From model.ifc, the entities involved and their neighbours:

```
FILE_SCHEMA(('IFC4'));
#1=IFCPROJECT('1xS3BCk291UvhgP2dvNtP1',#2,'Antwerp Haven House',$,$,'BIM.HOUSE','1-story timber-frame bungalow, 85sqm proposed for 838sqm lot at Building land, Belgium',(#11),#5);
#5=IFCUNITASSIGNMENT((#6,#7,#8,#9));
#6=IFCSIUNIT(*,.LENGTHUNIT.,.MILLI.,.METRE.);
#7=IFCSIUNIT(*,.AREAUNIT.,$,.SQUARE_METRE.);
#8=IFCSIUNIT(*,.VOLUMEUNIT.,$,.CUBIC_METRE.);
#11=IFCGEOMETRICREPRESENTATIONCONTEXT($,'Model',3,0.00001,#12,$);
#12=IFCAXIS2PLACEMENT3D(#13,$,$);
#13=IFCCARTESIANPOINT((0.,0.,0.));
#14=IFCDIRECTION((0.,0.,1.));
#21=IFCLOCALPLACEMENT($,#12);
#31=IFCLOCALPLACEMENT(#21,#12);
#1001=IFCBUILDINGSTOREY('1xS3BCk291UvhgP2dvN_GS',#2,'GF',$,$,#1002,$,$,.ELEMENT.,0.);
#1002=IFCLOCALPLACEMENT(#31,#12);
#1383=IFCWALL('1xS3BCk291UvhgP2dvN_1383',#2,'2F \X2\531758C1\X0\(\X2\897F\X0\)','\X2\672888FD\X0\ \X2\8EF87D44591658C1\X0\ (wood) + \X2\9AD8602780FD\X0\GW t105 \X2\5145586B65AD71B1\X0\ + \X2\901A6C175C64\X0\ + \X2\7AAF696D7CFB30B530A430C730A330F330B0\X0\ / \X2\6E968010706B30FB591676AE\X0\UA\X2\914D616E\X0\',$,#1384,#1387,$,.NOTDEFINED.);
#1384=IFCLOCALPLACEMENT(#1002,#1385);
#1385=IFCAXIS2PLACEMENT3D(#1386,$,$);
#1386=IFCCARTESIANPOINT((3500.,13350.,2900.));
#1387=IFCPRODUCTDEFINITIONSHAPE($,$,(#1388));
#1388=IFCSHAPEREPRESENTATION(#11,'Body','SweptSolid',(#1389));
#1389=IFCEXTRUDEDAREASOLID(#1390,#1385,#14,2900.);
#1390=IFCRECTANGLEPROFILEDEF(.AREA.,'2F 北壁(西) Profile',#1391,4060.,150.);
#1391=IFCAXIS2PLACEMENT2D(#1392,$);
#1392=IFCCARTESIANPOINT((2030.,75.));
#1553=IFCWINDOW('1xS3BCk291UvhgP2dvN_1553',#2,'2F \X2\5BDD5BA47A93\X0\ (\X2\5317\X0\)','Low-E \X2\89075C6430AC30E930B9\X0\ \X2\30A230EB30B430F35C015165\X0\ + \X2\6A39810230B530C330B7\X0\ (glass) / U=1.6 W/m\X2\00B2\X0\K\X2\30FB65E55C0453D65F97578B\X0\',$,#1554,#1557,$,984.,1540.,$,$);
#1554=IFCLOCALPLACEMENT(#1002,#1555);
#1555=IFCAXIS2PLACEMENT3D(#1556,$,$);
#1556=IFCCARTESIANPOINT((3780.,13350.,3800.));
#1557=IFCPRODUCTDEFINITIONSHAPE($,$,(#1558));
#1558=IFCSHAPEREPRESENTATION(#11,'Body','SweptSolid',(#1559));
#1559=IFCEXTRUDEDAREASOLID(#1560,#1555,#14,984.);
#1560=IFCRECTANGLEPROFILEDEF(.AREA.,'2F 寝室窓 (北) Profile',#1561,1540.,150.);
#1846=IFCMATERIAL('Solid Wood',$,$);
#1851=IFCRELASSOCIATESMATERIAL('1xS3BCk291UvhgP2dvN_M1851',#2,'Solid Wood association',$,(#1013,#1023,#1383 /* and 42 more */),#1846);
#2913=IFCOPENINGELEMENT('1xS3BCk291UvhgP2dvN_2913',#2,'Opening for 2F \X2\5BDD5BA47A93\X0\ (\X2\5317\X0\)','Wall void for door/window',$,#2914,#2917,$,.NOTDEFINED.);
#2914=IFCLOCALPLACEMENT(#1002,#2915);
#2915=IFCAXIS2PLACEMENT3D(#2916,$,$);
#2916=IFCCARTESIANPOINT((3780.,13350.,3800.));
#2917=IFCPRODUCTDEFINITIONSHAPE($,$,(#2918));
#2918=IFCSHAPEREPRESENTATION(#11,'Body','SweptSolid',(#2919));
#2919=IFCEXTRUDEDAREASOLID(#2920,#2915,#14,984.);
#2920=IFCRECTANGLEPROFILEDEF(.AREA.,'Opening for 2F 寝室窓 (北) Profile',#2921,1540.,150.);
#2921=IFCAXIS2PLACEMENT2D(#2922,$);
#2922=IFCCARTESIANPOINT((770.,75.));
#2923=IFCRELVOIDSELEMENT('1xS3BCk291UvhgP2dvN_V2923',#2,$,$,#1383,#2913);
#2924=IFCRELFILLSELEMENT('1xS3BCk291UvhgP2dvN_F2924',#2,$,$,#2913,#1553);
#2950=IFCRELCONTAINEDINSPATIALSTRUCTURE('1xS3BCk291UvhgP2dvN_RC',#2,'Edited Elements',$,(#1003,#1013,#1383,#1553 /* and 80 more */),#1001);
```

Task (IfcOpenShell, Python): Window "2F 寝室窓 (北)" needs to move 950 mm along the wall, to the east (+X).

```python
import ifcopenshell
import ifcopenshell.api.geometry
import ifcopenshell.util.placement
import ifcopenshell.util.unit

model = ifcopenshell.open("model.ifc")
unit_scale = ifcopenshell.util.unit.calculate_unit_scale(model)

window = model.by_guid("1xS3BCk291UvhgP2dvN_1553")
opening = window.FillsVoids[0].RelatingOpeningElement
wall = opening.VoidsElements[0].RelatingBuildingElement

wall_matrix = ifcopenshell.util.placement.get_local_placement(wall.ObjectPlacement)
shift = wall_matrix[:3, 0] * 0.95 / unit_scale
before = ifcopenshell.util.placement.get_local_placement(window.ObjectPlacement)[:3, 3].copy()

# The window is not placed relative to its opening, so move both.
for product in (opening, window):
    matrix = ifcopenshell.util.placement.get_local_placement(product.ObjectPlacement)
    matrix[:3, 3] += shift
    ifcopenshell.api.geometry.edit_object_placement(model, product=product, matrix=matrix, is_si=False)

after = ifcopenshell.util.placement.get_local_placement(window.ObjectPlacement)[:3, 3]
print("window moved by", (after - before).round(3) + 0.0)

model.write("model_rev.ifc")
```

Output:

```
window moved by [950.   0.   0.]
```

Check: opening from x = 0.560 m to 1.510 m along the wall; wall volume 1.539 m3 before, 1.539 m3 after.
